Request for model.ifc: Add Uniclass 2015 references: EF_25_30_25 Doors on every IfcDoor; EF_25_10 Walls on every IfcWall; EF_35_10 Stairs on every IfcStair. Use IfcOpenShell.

First a look at what the model holds.

```python
import ifcopenshell

model = ifcopenshell.open("model.ifc")
print(model.schema)
print("classifications:", [c.Name for c in model.by_type("IfcClassification")])
for ifc_class in ("IfcDoor", "IfcRoof", "IfcStair", "IfcWall", "IfcWindow"):
    print(ifc_class, len(model.by_type(ifc_class)))
```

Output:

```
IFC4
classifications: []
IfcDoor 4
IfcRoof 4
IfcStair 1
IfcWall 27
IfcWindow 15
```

```python
import ifcopenshell
import ifcopenshell.api.classification

model = ifcopenshell.open("model.ifc")

system = ifcopenshell.api.classification.add_classification(model, classification="Uniclass 2015")

codes = {
    "IfcDoor": ("EF_25_30_25", "Doors"),
    "IfcWall": ("EF_25_10", "Walls"),
    "IfcStair": ("EF_35_10", "Stairs"),
}
for ifc_class, (code, name) in codes.items():
    products = model.by_type(ifc_class)
    ifcopenshell.api.classification.add_reference(
        model, products=products, classification=system, identification=code, name=name
    )
    print(code, len(products))

model.write("model-out.ifc")
```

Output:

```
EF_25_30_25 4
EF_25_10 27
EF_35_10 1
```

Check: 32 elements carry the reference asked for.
